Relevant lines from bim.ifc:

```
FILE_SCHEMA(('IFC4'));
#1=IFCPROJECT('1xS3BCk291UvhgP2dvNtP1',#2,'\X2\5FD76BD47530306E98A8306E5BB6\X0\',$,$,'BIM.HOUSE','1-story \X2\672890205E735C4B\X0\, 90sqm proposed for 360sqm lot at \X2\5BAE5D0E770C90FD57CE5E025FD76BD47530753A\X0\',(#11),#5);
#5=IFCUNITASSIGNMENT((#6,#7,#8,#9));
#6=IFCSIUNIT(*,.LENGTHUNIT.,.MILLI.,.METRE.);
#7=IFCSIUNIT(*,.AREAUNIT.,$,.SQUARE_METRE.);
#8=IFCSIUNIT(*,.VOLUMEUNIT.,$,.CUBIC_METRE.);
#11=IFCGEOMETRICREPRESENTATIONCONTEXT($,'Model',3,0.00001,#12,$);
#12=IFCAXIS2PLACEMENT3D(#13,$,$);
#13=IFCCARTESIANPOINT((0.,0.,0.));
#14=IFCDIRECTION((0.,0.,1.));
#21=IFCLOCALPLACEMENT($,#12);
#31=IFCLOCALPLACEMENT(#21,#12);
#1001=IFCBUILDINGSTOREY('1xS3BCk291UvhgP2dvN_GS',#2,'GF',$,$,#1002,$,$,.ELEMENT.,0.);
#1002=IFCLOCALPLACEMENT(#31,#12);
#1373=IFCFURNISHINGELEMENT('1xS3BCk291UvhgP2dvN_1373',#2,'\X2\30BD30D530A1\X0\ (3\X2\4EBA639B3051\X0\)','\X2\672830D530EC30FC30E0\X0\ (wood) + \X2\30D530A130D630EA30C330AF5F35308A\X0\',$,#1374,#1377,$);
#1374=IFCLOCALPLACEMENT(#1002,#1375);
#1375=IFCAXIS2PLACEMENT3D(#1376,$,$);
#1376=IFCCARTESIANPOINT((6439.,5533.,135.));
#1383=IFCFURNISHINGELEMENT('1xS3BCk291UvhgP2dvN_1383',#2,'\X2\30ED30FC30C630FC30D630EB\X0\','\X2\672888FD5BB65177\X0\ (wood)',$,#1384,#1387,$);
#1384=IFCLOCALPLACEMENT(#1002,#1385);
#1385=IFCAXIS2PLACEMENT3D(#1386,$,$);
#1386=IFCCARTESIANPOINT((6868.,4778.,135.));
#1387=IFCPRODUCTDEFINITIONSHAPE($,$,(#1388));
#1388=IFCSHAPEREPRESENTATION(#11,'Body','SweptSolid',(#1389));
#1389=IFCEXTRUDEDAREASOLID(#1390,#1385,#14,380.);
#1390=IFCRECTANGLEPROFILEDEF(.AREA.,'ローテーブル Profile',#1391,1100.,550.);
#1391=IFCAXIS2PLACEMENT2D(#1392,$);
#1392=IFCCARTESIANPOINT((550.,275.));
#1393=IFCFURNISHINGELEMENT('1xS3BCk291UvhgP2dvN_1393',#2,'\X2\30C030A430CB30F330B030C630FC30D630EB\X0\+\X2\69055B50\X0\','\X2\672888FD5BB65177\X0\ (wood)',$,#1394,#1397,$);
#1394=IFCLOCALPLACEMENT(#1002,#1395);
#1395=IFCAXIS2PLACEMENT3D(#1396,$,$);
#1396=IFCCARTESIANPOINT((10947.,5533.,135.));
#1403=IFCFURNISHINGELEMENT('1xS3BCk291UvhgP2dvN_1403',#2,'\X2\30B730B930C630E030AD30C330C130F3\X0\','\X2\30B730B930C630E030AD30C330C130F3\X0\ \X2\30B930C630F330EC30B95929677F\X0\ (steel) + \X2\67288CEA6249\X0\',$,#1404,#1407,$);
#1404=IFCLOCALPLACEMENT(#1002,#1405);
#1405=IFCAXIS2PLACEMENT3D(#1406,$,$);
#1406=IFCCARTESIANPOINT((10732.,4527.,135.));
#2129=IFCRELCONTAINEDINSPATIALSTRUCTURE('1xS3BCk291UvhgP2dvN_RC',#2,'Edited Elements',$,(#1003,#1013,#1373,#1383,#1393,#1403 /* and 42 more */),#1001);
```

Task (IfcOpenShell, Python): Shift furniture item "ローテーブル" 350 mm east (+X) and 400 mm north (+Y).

```python
import ifcopenshell
import ifcopenshell.api.geometry
import ifcopenshell.util.placement
import ifcopenshell.util.unit

model = ifcopenshell.open("bim.ifc")
unit_scale = ifcopenshell.util.unit.calculate_unit_scale(model)

item = model.by_id(1383)
matrix = ifcopenshell.util.placement.get_local_placement(item.ObjectPlacement)
matrix[0, 3] += 0.35 / unit_scale
matrix[1, 3] += 0.4 / unit_scale
ifcopenshell.api.geometry.edit_object_placement(model, product=item, matrix=matrix, is_si=False)

print(ifcopenshell.util.placement.get_local_placement(item.ObjectPlacement).round(3) + 0.0)

model.write("bim_rev.ifc")
```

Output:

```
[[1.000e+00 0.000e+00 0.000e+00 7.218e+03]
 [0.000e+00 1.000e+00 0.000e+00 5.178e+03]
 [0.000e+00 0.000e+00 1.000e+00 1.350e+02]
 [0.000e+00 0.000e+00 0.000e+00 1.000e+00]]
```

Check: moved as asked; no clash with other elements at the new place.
